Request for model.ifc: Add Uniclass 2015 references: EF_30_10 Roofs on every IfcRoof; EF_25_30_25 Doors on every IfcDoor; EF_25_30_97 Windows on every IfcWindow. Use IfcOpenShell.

First a look at what the model holds.

```python
import ifcopenshell

model = ifcopenshell.open("model.ifc")
print(model.schema)
print("classifications:", [c.Name for c in model.by_type("IfcClassification")])
for ifc_class in ("IfcDoor", "IfcRoof", "IfcStair", "IfcWall", "IfcWindow"):
    print(ifc_class, len(model.by_type(ifc_class)))
```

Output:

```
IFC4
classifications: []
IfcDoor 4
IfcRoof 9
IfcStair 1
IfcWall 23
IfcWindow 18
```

```python
import ifcopenshell
import ifcopenshell.api.classification

model = ifcopenshell.open("model.ifc")

system = ifcopenshell.api.classification.add_classification(model, classification="Uniclass 2015")

codes = {
    "IfcRoof": ("EF_30_10", "Roofs"),
    "IfcDoor": ("EF_25_30_25", "Doors"),
    "IfcWindow": ("EF_25_30_97", "Windows"),
}
for ifc_class, (code, name) in codes.items():
    products = model.by_type(ifc_class)
    ifcopenshell.api.classification.add_reference(
        model, products=products, classification=system, identification=code, name=name
    )
    print(code, len(products))

model.write("model_rev.ifc")
```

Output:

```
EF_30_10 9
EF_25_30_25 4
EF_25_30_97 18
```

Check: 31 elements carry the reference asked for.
